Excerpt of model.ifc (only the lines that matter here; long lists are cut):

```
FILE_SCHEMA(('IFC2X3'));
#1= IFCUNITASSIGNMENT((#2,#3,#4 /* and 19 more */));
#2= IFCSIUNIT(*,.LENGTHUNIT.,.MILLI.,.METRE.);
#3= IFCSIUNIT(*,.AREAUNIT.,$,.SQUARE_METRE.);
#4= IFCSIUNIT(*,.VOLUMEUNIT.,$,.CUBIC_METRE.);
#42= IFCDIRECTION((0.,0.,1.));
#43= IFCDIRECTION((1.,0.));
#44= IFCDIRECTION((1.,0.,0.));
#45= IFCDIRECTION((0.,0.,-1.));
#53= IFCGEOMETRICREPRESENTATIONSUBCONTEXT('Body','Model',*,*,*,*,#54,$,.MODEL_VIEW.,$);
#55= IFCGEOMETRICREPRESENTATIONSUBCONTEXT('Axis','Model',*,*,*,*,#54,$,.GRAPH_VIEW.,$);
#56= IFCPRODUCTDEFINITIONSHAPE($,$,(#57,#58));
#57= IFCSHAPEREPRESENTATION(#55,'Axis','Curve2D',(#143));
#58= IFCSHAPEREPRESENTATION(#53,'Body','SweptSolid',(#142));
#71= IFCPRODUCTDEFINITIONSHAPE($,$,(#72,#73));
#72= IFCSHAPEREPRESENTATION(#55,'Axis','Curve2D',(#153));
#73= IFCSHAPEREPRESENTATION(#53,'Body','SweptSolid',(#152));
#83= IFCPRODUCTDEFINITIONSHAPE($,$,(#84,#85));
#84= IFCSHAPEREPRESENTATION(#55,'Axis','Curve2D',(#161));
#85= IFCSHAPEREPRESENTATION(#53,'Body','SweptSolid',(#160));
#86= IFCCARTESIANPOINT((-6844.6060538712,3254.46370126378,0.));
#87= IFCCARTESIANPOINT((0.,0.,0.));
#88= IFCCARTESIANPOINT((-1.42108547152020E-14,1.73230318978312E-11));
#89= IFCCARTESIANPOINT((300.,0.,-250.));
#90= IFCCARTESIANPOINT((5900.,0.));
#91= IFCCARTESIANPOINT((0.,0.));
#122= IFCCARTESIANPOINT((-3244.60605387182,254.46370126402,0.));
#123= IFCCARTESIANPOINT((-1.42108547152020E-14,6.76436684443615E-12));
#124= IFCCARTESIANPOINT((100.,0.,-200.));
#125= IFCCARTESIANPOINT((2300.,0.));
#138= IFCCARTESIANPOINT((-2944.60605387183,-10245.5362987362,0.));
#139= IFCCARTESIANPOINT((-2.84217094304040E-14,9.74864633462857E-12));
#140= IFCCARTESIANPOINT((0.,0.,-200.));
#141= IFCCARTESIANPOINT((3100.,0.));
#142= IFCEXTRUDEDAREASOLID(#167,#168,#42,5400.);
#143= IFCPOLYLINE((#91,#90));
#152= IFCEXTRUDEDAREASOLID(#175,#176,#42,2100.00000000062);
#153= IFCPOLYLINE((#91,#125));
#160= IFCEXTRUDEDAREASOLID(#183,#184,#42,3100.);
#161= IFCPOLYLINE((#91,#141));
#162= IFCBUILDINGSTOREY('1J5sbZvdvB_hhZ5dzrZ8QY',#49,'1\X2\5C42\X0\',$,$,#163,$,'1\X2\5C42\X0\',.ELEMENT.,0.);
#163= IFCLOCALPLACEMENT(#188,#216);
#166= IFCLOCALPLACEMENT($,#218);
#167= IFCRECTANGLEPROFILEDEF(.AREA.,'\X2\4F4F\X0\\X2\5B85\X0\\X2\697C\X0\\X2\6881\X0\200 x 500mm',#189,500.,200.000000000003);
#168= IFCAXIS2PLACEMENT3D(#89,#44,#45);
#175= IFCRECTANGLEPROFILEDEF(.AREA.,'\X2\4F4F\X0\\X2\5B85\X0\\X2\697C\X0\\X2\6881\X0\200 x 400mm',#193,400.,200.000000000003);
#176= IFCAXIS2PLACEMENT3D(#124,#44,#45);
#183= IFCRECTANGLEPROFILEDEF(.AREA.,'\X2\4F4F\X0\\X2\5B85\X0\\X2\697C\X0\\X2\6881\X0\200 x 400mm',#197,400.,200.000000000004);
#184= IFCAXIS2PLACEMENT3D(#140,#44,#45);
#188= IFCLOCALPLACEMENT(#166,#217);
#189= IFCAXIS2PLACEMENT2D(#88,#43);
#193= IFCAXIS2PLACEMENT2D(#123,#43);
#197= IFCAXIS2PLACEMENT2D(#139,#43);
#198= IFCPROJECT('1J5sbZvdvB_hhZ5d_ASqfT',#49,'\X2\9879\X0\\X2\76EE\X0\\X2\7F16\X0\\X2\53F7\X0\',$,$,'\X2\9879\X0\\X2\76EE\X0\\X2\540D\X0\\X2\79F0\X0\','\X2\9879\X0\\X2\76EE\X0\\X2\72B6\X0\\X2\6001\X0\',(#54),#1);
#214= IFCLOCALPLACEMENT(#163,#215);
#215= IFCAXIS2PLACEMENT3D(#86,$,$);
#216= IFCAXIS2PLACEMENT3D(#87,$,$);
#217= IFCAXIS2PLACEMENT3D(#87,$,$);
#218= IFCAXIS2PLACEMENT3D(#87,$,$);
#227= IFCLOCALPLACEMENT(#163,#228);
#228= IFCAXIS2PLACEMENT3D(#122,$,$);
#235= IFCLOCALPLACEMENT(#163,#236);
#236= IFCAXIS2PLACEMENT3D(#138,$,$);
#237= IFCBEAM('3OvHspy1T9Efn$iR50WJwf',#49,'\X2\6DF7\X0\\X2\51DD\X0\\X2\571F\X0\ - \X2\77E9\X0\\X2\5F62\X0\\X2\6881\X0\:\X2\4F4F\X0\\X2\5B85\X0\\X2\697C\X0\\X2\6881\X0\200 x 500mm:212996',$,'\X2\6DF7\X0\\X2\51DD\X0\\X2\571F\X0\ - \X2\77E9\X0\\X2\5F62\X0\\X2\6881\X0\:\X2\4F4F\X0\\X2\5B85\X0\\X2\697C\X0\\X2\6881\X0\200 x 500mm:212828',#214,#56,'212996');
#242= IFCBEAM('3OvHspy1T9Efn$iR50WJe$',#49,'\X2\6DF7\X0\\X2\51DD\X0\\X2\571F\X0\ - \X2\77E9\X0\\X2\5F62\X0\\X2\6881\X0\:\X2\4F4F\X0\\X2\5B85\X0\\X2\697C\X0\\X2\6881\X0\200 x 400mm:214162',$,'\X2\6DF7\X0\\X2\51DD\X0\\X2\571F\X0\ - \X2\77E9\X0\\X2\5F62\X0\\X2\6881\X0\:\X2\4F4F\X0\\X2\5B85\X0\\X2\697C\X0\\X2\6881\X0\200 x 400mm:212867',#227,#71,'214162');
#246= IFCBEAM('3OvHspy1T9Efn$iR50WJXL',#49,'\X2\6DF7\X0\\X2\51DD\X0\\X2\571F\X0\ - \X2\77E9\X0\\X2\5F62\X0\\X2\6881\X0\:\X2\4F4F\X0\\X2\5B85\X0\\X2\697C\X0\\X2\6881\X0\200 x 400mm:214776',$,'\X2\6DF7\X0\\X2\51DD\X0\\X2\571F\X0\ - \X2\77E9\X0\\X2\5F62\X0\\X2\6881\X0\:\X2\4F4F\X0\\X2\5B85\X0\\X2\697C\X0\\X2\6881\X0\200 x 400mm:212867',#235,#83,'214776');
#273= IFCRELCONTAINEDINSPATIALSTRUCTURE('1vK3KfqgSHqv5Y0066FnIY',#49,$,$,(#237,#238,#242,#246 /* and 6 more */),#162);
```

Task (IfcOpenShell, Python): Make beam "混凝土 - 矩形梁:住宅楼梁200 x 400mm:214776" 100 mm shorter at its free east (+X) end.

```python
import numpy as np
import ifcopenshell
import ifcopenshell.util.representation
import ifcopenshell.util.unit

model = ifcopenshell.open("model.ifc")
unit_scale = ifcopenshell.util.unit.calculate_unit_scale(model)

member = model.by_guid("3OvHspy1T9Efn$iR50WJXL")
change = -0.1 / unit_scale

# The extrusion runs towards the end named, so only its depth changes.
body = ifcopenshell.util.representation.get_representation(member, "Model", "Body")
solid = body.Items[0]
old_length = solid.Depth
solid.Depth += change

# Move the axis end point with it.
axis = next(r for r in member.Representation.Representations if r.RepresentationIdentifier == "Axis").Items[0]
start, end = (np.array(p.Coordinates) for p in axis.Points)
end = end + (end - start) / np.linalg.norm(end - start) * change
point = model.createIfcCartesianPoint(end.tolist())
axis.Points = [axis.Points[0], point]

print(f"length {old_length:g} -> {solid.Depth:g}")

model.write("model_rev.ifc")
```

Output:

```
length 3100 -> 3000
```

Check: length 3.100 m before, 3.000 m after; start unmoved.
